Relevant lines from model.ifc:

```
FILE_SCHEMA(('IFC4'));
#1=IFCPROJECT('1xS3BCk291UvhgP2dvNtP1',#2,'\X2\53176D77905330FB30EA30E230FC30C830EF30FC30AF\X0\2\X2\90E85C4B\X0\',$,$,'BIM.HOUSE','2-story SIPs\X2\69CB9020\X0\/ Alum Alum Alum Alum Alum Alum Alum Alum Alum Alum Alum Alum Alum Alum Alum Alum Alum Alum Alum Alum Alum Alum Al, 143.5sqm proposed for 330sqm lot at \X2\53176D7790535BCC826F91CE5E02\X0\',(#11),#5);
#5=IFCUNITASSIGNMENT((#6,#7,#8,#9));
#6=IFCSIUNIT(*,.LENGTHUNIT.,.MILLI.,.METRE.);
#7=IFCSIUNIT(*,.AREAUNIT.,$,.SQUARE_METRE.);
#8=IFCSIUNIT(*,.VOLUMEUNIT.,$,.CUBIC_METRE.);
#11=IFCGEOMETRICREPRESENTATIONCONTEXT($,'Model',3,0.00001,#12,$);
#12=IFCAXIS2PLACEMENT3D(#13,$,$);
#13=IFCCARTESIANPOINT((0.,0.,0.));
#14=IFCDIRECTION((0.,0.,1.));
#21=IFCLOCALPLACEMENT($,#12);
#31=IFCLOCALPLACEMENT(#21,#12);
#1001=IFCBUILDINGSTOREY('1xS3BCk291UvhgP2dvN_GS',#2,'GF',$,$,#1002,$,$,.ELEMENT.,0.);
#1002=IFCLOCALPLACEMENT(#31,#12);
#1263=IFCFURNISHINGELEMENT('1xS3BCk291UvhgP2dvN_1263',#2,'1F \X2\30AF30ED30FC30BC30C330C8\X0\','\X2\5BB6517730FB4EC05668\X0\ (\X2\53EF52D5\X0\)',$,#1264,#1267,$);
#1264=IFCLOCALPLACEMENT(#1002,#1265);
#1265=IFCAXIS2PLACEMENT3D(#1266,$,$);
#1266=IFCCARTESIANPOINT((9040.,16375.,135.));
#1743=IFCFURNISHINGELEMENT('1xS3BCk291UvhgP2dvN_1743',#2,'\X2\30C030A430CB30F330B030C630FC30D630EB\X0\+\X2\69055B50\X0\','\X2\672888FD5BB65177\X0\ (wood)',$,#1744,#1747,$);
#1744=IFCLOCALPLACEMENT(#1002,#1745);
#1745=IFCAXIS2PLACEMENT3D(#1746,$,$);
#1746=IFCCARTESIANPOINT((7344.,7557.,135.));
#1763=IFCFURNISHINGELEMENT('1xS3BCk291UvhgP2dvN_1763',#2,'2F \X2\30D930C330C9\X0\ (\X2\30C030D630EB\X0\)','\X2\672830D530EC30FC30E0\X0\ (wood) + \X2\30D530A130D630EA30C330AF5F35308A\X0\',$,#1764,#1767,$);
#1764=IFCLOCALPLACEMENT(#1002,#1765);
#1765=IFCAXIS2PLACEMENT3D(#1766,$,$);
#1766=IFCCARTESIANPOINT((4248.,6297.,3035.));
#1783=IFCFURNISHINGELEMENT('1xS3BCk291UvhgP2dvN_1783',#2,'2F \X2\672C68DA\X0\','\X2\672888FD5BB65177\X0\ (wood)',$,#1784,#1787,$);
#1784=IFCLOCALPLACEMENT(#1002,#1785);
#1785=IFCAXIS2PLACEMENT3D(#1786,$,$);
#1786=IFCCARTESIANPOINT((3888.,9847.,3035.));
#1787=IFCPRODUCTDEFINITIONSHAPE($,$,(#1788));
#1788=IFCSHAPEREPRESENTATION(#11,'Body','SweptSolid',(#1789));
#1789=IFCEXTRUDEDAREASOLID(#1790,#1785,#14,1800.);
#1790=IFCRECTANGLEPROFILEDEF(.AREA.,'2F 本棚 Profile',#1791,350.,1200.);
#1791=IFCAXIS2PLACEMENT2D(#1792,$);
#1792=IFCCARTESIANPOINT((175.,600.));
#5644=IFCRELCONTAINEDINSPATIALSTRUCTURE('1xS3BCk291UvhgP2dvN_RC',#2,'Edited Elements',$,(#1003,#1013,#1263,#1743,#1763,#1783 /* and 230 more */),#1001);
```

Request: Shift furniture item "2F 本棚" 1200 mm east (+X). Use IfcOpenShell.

```python
import ifcopenshell
import ifcopenshell.api.geometry
import ifcopenshell.util.placement
import ifcopenshell.util.unit

model = ifcopenshell.open("model.ifc")
unit_scale = ifcopenshell.util.unit.calculate_unit_scale(model)

item = model.by_guid("1xS3BCk291UvhgP2dvN_1783")
matrix = ifcopenshell.util.placement.get_local_placement(item.ObjectPlacement)
matrix[0, 3] += 1.2 / unit_scale
ifcopenshell.api.geometry.edit_object_placement(model, product=item, matrix=matrix, is_si=False)

print(ifcopenshell.util.placement.get_local_placement(item.ObjectPlacement).round(3) + 0.0)

model.write("model_edited.ifc")
```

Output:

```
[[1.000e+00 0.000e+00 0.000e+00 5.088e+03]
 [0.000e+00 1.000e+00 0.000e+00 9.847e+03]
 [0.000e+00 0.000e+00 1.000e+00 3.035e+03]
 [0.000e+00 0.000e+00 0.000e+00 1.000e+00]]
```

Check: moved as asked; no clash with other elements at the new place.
